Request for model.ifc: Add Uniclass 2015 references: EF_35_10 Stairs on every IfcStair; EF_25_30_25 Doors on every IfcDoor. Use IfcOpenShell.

First a look at what the model holds.

```python
import ifcopenshell

model = ifcopenshell.open("model.ifc")
print(model.schema)
print("classifications:", [c.Name for c in model.by_type("IfcClassification")])
for ifc_class in ("IfcDoor", "IfcRoof", "IfcStair", "IfcWall", "IfcWindow"):
    print(ifc_class, len(model.by_type(ifc_class)))
```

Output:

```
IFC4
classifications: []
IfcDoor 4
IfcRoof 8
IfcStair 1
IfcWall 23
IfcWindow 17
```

```python
import ifcopenshell
import ifcopenshell.api.classification

model = ifcopenshell.open("model.ifc")

system = ifcopenshell.api.classification.add_classification(model, classification="Uniclass 2015")

codes = {
    "IfcStair": ("EF_35_10", "Stairs"),
    "IfcDoor": ("EF_25_30_25", "Doors"),
}
for ifc_class, (code, name) in codes.items():
    products = model.by_type(ifc_class)
    ifcopenshell.api.classification.add_reference(
        model, products=products, classification=system, identification=code, name=name
    )
    print(code, len(products))

model.write("model_v2.ifc")
```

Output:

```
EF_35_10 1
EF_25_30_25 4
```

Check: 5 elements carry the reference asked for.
